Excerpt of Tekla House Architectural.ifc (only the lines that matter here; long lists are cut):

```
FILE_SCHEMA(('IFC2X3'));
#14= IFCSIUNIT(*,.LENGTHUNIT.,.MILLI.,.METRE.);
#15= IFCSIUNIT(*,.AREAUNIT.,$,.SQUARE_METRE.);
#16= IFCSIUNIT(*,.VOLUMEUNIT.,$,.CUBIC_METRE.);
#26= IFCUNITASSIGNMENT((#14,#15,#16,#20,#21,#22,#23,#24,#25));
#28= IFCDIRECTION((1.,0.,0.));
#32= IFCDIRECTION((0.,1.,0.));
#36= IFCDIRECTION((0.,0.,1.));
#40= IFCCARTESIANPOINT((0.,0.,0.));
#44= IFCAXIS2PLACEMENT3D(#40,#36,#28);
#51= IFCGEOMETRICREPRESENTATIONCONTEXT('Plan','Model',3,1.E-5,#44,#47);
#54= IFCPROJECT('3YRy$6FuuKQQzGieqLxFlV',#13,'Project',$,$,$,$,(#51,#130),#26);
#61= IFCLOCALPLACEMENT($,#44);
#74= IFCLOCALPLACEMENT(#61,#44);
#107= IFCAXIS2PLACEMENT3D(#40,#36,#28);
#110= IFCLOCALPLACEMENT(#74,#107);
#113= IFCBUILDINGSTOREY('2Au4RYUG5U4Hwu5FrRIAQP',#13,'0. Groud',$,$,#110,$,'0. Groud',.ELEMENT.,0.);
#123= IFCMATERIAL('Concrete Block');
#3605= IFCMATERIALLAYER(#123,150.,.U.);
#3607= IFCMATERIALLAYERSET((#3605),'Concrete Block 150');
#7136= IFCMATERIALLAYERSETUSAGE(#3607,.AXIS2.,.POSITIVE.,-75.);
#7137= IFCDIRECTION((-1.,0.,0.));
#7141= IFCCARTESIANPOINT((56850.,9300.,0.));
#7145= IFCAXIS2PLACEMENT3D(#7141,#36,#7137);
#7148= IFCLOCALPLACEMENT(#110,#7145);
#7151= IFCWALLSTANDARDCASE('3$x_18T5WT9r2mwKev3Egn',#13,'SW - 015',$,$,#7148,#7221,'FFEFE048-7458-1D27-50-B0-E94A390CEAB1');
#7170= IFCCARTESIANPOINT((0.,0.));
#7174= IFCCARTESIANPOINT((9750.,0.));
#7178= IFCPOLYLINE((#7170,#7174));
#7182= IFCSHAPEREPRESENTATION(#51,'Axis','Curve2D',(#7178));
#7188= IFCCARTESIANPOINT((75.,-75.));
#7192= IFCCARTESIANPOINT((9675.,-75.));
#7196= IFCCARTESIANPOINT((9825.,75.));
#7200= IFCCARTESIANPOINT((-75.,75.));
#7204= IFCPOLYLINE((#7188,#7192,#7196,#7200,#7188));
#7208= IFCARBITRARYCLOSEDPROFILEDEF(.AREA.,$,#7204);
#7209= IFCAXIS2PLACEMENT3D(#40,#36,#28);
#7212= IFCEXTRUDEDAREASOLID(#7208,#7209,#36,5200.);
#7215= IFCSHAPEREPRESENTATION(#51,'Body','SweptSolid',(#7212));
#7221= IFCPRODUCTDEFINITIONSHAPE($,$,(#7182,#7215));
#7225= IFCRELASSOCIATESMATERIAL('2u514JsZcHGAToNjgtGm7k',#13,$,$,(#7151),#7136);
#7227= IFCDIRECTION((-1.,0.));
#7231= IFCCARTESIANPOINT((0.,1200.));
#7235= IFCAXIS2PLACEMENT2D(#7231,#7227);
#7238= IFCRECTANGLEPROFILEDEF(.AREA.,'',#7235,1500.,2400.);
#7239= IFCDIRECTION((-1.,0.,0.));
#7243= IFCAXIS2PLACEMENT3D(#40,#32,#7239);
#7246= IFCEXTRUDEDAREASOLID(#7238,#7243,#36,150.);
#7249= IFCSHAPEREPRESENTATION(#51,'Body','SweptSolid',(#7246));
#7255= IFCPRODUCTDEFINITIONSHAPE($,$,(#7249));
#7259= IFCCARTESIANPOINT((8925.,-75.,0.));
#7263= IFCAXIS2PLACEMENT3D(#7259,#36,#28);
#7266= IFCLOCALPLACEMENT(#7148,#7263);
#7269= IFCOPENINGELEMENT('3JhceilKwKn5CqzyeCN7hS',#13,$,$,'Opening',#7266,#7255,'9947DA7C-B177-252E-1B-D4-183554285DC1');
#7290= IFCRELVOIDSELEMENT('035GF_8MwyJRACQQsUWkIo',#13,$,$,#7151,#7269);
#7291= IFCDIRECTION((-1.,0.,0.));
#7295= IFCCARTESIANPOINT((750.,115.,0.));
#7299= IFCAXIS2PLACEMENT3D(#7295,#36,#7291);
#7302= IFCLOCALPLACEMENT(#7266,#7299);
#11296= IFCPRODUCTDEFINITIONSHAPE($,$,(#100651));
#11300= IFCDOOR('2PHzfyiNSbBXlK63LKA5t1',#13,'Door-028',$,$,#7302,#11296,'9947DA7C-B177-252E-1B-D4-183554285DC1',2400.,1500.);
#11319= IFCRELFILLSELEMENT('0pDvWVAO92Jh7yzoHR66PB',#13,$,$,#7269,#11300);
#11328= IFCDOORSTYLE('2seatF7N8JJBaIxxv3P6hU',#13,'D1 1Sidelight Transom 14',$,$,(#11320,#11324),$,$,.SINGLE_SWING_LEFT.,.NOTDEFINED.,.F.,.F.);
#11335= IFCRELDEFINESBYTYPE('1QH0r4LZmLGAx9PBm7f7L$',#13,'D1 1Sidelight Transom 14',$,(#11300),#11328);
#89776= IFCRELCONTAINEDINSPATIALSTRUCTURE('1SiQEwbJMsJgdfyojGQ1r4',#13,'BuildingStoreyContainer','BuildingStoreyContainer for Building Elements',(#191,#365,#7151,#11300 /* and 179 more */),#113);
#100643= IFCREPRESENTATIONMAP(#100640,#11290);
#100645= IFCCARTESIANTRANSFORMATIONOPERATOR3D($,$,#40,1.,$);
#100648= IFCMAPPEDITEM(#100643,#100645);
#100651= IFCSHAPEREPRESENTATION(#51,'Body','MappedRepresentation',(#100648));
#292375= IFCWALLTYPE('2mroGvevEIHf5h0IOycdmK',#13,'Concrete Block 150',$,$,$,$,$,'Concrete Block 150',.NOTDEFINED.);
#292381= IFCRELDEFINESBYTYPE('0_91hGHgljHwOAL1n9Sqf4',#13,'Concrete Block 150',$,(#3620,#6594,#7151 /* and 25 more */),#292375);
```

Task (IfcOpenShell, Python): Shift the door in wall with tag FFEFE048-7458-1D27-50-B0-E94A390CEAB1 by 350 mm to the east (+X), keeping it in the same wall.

```python
import ifcopenshell
import ifcopenshell.api.geometry
import ifcopenshell.util.placement
import ifcopenshell.util.unit

model = ifcopenshell.open("Tekla House Architectural.ifc")
unit_scale = ifcopenshell.util.unit.calculate_unit_scale(model)

door = model.by_guid("2PHzfyiNSbBXlK63LKA5t1")
opening = door.FillsVoids[0].RelatingOpeningElement
wall = opening.VoidsElements[0].RelatingBuildingElement

wall_matrix = ifcopenshell.util.placement.get_local_placement(wall.ObjectPlacement)
shift = wall_matrix[:3, 0] * -0.35 / unit_scale
before = ifcopenshell.util.placement.get_local_placement(door.ObjectPlacement)[:3, 3].copy()

# The door is placed relative to its opening, so it follows when the opening moves.
matrix = ifcopenshell.util.placement.get_local_placement(opening.ObjectPlacement)
matrix[:3, 3] += shift
ifcopenshell.api.geometry.edit_object_placement(
    model, product=opening, matrix=matrix, is_si=False, should_transform_children=True
)

after = ifcopenshell.util.placement.get_local_placement(door.ObjectPlacement)[:3, 3]
print("door moved by", (after - before).round(3) + 0.0)

model.write("Tekla House Architectural_rev.ifc")
```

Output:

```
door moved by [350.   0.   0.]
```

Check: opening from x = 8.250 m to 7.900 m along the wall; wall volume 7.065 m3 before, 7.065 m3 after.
